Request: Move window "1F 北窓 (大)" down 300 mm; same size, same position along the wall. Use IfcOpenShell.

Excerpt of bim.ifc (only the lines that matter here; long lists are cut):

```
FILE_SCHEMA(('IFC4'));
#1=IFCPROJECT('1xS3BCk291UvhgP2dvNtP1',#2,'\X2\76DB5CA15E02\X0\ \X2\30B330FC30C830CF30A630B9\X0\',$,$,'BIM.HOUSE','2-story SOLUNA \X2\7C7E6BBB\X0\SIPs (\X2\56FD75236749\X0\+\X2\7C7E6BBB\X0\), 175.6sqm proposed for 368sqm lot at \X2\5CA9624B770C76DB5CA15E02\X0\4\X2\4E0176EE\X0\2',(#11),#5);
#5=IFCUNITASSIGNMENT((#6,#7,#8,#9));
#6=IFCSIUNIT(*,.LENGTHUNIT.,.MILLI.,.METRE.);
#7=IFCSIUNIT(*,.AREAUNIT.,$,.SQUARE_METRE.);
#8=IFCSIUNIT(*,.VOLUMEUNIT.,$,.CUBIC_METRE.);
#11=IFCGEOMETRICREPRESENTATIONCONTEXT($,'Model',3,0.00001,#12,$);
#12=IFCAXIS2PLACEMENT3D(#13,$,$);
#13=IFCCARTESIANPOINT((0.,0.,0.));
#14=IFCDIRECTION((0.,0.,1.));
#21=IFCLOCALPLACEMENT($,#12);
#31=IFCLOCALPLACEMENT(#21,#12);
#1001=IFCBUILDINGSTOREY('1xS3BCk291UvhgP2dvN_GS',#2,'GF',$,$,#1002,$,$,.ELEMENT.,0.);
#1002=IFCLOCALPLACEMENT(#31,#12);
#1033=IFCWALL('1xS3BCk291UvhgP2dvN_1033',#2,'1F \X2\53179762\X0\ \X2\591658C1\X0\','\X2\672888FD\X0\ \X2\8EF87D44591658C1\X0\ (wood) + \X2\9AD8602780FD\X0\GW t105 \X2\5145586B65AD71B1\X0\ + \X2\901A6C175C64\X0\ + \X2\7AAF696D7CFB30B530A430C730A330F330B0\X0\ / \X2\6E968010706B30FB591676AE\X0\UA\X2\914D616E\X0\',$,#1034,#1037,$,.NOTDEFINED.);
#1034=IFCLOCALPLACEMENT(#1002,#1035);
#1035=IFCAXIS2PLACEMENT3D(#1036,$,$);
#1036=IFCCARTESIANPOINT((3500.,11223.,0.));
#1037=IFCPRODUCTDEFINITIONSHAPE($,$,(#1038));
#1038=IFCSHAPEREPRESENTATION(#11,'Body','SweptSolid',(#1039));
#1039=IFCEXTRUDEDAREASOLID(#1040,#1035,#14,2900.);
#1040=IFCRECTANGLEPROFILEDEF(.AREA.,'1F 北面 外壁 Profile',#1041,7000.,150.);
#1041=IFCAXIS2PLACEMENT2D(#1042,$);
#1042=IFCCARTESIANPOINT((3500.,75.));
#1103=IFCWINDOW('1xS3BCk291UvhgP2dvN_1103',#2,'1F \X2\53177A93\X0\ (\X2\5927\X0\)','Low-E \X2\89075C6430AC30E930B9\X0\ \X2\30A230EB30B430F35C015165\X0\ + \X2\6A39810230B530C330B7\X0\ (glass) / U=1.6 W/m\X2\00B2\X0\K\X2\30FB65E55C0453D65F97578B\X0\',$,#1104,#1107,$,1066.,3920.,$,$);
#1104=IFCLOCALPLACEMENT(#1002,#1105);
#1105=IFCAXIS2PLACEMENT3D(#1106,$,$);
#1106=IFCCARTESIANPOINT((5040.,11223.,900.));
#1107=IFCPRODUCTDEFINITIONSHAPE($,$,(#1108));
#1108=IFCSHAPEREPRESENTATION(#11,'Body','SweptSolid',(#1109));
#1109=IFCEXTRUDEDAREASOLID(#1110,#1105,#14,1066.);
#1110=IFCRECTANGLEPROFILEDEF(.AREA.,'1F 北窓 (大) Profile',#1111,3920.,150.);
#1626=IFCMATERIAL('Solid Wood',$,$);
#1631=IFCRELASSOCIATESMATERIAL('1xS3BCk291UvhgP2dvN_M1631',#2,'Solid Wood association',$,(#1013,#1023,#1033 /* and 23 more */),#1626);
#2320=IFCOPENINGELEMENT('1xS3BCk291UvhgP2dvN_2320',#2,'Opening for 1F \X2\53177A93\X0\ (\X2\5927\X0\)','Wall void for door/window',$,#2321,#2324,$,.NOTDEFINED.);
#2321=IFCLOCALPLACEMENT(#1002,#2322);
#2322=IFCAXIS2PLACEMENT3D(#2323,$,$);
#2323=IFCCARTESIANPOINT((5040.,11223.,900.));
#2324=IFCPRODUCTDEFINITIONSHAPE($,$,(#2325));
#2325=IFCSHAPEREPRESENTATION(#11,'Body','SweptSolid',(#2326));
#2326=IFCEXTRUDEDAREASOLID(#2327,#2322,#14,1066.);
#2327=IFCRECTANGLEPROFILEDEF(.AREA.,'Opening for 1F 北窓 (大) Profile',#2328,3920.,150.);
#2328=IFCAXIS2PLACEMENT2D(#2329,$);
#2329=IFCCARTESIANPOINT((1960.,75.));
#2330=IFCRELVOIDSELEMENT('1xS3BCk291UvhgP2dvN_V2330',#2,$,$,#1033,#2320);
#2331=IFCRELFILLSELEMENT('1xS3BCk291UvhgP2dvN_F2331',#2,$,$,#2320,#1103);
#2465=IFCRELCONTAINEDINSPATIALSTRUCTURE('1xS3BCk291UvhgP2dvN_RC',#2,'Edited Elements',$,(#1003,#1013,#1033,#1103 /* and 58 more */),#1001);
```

```python
import numpy as np
import ifcopenshell
import ifcopenshell.api.geometry
import ifcopenshell.util.placement
import ifcopenshell.util.unit

model = ifcopenshell.open("bim.ifc")
unit_scale = ifcopenshell.util.unit.calculate_unit_scale(model)

window = model.by_id(1103)
opening = window.FillsVoids[0].RelatingOpeningElement
dz = -0.3 / unit_scale

shift = np.array([0.0, 0.0, dz])
# The window is not placed relative to its opening, so move both.
for product in (opening, window):
    matrix = ifcopenshell.util.placement.get_local_placement(product.ObjectPlacement)
    matrix[:3, 3] += shift
    ifcopenshell.api.geometry.edit_object_placement(model, product=product, matrix=matrix, is_si=False)

print(f"moved by {dz * unit_scale:+.3f} m")

model.write("bim-out.ifc")
```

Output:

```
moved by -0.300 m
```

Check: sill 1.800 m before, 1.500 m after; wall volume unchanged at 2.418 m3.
